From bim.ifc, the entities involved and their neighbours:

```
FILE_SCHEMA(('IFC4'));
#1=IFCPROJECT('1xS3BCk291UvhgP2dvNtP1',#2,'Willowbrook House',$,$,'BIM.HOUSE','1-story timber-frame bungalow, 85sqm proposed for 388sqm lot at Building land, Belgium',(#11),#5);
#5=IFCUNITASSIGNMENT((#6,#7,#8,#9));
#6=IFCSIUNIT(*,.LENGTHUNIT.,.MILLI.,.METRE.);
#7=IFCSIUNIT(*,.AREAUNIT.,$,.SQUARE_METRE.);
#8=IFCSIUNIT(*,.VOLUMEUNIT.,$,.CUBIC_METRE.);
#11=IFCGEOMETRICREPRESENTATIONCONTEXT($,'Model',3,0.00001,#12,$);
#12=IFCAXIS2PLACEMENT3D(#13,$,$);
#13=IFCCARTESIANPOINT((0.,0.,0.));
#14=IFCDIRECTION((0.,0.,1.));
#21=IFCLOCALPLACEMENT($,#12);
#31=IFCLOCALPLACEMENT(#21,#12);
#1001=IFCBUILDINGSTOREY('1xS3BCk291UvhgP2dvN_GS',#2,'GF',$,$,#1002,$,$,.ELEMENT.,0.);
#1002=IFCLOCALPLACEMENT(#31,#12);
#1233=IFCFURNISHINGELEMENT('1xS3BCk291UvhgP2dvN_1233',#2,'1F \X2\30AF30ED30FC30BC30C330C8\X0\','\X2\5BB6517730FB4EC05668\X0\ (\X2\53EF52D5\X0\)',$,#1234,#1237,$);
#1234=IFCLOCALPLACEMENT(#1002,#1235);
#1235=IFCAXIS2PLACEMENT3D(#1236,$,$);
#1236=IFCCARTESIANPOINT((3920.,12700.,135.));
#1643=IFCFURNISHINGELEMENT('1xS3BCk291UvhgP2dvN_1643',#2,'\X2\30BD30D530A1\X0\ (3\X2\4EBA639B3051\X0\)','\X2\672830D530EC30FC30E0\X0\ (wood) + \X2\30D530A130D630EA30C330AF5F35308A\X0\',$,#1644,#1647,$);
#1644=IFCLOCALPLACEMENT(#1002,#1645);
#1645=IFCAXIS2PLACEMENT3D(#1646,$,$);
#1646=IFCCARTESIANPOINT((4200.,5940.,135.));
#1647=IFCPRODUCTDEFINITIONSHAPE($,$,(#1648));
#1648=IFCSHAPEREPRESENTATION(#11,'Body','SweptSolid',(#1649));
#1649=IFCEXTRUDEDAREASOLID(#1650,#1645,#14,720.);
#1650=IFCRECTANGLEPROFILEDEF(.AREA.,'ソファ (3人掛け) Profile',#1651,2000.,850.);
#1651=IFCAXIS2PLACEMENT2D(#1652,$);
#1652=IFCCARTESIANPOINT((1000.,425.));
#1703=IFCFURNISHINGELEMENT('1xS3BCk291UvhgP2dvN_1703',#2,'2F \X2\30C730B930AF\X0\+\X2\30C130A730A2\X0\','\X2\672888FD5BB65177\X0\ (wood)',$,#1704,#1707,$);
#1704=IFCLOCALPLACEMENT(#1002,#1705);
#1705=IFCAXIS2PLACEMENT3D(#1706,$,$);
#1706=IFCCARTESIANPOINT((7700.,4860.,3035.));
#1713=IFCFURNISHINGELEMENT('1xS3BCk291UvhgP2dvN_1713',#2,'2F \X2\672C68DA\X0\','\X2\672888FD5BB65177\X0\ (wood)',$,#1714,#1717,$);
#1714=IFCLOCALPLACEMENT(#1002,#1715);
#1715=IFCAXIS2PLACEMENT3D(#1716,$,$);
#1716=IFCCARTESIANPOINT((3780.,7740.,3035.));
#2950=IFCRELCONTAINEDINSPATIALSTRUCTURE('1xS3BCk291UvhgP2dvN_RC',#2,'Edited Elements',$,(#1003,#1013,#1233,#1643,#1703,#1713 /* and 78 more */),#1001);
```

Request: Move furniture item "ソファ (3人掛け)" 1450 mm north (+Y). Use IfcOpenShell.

```python
import ifcopenshell
import ifcopenshell.api.geometry
import ifcopenshell.util.placement

model = ifcopenshell.open("bim.ifc")

item = model.by_guid("1xS3BCk291UvhgP2dvN_1643")
matrix = ifcopenshell.util.placement.get_local_placement(item.ObjectPlacement)
matrix[1, 3] += 1450.0
ifcopenshell.api.geometry.edit_object_placement(model, product=item, matrix=matrix, is_si=False)

print(ifcopenshell.util.placement.get_local_placement(item.ObjectPlacement).round(3) + 0.0)

model.write("bim-out.ifc")
```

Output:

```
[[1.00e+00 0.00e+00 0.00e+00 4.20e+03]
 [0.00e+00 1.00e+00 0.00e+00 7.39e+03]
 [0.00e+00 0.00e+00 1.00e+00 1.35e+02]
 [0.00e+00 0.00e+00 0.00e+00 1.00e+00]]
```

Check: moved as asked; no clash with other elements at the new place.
